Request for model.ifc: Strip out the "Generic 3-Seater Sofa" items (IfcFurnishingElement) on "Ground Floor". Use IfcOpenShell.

First a look at what the model holds.

```python
import ifcopenshell
import ifcopenshell.util.element

model = ifcopenshell.open("model.ifc")
print(model.schema)
storey = next(s for s in model.by_type("IfcBuildingStorey") if s.Name == "Ground Floor")
furniture = [e for e in ifcopenshell.util.element.get_decomposition(storey) if e.is_a("IfcFurnishingElement")]
seen = {}
for e in furniture:
    element_type = ifcopenshell.util.element.get_type(e)
    name = element_type.Name if element_type not in (None, e) else None
    seen[name] = seen.get(name, 0) + 1
for name, count in sorted(seen.items(), key=str):
    print(count, "x", name)
```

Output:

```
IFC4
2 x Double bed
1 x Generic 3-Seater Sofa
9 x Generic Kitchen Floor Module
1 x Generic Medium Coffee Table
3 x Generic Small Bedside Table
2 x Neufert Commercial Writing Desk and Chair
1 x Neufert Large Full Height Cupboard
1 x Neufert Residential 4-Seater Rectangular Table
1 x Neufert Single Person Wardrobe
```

```python
import ifcopenshell
import ifcopenshell.api.root
import ifcopenshell.util.element

model = ifcopenshell.open("model.ifc")

storey = next(s for s in model.by_type("IfcBuildingStorey") if s.Name == "Ground Floor")
furniture = [e for e in ifcopenshell.util.element.get_decomposition(storey) if e.is_a("IfcFurnishingElement")]
targets = [e for e in furniture if (t := ifcopenshell.util.element.get_type(e)) not in (None, e) and t.Name == "Generic 3-Seater Sofa"]

for e in targets:
    ifcopenshell.api.root.remove_product(model, product=e)
print(len(targets), "removed")

model.write("model_v2.ifc")
```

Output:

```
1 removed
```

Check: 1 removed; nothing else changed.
